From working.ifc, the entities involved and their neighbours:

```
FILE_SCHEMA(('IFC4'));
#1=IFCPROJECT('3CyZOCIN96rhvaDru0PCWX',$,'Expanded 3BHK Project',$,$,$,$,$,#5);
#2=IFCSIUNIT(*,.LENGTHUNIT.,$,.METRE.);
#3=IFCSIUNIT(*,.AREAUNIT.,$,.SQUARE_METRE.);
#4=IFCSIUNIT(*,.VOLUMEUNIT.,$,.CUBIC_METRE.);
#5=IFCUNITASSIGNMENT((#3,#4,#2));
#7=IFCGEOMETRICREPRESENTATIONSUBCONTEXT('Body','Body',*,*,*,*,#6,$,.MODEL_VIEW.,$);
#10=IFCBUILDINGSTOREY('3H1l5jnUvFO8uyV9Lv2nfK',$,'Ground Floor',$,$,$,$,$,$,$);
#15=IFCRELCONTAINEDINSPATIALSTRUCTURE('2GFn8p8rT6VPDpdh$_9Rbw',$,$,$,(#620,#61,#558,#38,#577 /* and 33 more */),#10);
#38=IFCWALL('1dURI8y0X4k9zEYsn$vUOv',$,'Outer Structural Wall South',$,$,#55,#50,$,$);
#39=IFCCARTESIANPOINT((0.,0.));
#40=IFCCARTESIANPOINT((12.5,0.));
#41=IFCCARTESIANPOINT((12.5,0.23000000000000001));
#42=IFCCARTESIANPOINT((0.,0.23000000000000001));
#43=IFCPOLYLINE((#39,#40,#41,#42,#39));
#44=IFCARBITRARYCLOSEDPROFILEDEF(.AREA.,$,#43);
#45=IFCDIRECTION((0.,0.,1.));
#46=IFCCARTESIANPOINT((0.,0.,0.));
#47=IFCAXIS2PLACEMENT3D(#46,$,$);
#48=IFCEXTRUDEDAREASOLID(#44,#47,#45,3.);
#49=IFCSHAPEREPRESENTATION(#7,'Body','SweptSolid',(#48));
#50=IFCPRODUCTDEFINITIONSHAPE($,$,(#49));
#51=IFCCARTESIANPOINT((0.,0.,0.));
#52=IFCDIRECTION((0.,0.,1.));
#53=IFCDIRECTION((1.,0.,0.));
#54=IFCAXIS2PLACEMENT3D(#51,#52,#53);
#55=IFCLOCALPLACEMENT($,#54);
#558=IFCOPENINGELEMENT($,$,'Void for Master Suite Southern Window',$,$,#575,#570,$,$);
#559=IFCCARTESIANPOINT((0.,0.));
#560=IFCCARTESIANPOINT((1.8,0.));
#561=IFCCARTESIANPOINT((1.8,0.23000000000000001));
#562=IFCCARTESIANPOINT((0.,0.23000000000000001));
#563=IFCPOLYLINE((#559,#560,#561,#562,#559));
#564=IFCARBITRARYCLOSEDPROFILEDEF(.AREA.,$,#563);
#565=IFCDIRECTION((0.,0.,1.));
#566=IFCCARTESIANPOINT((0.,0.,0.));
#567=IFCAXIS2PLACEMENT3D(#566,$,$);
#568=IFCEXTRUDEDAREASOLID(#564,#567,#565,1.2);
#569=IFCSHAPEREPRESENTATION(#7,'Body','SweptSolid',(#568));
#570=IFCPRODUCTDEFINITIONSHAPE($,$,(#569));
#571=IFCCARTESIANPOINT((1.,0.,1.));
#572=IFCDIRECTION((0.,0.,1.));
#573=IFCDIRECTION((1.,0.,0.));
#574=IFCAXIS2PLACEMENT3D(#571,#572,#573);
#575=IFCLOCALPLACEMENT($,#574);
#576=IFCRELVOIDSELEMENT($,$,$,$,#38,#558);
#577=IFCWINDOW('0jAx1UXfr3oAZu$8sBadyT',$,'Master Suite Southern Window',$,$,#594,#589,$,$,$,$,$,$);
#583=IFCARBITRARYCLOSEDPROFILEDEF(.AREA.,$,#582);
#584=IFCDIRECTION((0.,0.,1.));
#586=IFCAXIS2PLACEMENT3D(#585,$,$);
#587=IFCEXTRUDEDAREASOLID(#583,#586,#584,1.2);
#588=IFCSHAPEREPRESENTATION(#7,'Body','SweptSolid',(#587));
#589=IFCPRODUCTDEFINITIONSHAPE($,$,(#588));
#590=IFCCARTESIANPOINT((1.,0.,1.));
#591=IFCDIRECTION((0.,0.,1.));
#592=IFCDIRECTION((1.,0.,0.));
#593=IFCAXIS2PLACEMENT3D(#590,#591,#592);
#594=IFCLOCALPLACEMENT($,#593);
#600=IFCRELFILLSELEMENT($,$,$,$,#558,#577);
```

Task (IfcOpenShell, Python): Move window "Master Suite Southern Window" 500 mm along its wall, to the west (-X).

```python
import ifcopenshell
import ifcopenshell.api.geometry
import ifcopenshell.util.placement

model = ifcopenshell.open("working.ifc")

window = model.by_guid("0jAx1UXfr3oAZu$8sBadyT")
opening = window.FillsVoids[0].RelatingOpeningElement
wall = opening.VoidsElements[0].RelatingBuildingElement

wall_matrix = ifcopenshell.util.placement.get_local_placement(wall.ObjectPlacement)
shift = wall_matrix[:3, 0] * -0.5
before = ifcopenshell.util.placement.get_local_placement(window.ObjectPlacement)[:3, 3].copy()

# The window is not placed relative to its opening, so move both.
for product in (opening, window):
    matrix = ifcopenshell.util.placement.get_local_placement(product.ObjectPlacement)
    matrix[:3, 3] += shift
    ifcopenshell.api.geometry.edit_object_placement(model, product=product, matrix=matrix, is_si=False)

after = ifcopenshell.util.placement.get_local_placement(window.ObjectPlacement)[:3, 3]
print("window moved by", (after - before).round(3) + 0.0)

model.write("working-out.ifc")
```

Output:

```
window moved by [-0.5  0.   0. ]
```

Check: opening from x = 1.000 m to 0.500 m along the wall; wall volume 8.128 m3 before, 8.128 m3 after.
